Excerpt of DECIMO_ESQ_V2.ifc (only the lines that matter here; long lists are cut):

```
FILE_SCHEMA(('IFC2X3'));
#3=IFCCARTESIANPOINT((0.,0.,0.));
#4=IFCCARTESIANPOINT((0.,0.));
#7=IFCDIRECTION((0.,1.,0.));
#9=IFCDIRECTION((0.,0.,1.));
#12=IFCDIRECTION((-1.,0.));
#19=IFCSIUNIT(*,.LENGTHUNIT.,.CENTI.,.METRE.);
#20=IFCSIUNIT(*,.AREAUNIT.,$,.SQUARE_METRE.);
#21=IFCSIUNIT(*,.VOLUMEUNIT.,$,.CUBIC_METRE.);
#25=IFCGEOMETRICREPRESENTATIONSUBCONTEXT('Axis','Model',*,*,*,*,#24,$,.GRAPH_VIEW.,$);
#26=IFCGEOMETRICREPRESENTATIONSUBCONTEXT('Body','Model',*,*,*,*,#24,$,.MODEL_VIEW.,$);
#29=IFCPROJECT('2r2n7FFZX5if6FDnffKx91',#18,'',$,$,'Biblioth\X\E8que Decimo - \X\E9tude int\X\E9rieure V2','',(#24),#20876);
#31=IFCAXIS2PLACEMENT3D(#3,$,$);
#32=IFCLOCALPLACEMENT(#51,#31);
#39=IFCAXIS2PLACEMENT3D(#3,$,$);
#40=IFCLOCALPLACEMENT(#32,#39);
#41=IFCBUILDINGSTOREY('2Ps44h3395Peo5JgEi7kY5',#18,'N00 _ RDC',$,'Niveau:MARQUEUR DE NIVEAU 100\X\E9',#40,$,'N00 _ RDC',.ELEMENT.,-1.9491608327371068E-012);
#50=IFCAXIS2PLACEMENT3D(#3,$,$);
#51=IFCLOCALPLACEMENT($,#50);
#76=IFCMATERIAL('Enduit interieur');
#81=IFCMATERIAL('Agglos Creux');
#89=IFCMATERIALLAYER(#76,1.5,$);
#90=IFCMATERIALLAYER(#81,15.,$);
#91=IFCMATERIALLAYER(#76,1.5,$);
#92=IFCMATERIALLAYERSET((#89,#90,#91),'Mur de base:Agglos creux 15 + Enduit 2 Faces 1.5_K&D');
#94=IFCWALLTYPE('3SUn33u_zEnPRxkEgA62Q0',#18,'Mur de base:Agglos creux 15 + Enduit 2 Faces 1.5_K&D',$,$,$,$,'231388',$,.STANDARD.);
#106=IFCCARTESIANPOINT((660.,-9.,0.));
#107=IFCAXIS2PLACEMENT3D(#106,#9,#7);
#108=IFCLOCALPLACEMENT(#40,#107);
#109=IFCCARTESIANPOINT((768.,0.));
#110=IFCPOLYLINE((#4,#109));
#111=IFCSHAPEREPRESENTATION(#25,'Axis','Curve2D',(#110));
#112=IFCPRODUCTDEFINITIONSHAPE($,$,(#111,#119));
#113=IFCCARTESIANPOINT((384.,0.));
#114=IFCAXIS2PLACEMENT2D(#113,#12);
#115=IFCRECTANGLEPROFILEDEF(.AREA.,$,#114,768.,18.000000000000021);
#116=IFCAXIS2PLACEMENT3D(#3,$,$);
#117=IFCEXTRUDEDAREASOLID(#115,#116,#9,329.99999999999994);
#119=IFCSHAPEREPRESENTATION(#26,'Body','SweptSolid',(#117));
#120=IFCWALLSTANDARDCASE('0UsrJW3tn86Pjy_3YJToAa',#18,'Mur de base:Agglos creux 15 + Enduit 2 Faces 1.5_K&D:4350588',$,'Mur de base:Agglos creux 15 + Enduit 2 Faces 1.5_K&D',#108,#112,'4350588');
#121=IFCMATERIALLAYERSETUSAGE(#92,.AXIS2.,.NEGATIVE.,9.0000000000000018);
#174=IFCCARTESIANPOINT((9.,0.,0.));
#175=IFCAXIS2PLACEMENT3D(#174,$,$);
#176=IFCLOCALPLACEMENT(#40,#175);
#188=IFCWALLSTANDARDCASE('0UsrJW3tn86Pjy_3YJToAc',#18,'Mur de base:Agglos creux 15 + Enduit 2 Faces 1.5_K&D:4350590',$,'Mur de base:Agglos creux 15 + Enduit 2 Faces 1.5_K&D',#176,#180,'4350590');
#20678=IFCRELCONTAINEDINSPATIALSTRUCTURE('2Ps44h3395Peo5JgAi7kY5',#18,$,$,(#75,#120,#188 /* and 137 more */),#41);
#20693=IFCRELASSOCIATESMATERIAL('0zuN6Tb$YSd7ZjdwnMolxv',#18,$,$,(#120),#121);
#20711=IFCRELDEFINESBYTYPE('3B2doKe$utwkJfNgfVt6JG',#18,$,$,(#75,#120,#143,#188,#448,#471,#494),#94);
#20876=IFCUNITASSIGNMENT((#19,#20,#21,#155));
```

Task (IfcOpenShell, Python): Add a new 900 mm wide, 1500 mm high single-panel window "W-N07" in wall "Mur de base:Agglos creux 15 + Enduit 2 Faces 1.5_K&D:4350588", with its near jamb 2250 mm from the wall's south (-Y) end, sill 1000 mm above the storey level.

```python
import numpy as np
import ifcopenshell
import ifcopenshell.api.feature
import ifcopenshell.api.geometry
import ifcopenshell.api.root
import ifcopenshell.api.spatial
import ifcopenshell.api.type
import ifcopenshell.geom
import ifcopenshell.util.element
import ifcopenshell.util.placement
import ifcopenshell.util.representation
import ifcopenshell.util.shape
import ifcopenshell.util.unit

model = ifcopenshell.open("DECIMO_ESQ_V2.ifc")
unit_scale = ifcopenshell.util.unit.calculate_unit_scale(model)
settings = ifcopenshell.geom.settings()


def volume(element):
    """Net volume in cubic metres, openings subtracted."""
    shape = ifcopenshell.geom.create_shape(settings, element)
    return ifcopenshell.util.shape.get_volume(shape.geometry)


wall = model.by_guid("0UsrJW3tn86Pjy_3YJToAa")
storey = ifcopenshell.util.element.get_container(wall, ifc_class="IfcBuildingStorey")
context = ifcopenshell.util.representation.get_context(model, "Model", "Body", "MODEL_VIEW")
before = volume(wall)

width, height, from_end, sill = 0.9, 1.5, 2.25, 1  # metres

# The wall runs along its own X axis, and the end named is its -X end.
wall_shape = ifcopenshell.geom.create_shape(settings, wall)
x, y, z = ifcopenshell.util.shape.get_vertices(wall_shape.geometry).T
start = x.min() + from_end
face, thickness = float(y.min()), float(y.max() - y.min())
wall_matrix = ifcopenshell.util.placement.get_local_placement(wall.ObjectPlacement)
level = ifcopenshell.util.placement.get_local_placement(storey.ObjectPlacement)[2, 3]


def in_wall(x, y):
    """Placement at x, y metres in the wall's axes, at sill height."""
    matrix = wall_matrix.copy()
    matrix[:, 3] = wall_matrix @ np.array([x / unit_scale, y / unit_scale, 0.0, 1.0])
    matrix[2, 3] = level + sill / unit_scale
    return matrix


# Opening: a box that overshoots both wall faces by 50 mm.
opening = ifcopenshell.api.root.create_entity(model, ifc_class="IfcOpeningElement")
box = ifcopenshell.api.geometry.add_wall_representation(
    model, context=context, length=width, height=height, thickness=thickness + 0.1
)
ifcopenshell.api.geometry.assign_representation(model, product=opening, representation=box)
ifcopenshell.api.geometry.edit_object_placement(model, product=opening, matrix=in_wall(start, face - 0.05), is_si=False)
ifcopenshell.api.feature.add_feature(model, feature=opening, element=wall)

window = ifcopenshell.api.root.create_entity(model, ifc_class="IfcWindow", name="W-N07")
window.OverallWidth, window.OverallHeight = width / unit_scale, height / unit_scale
body = ifcopenshell.api.geometry.add_window_representation(
    model,
    context=context,
    overall_width=window.OverallWidth,
    overall_height=window.OverallHeight,
    partition_type="SINGLE_PANEL",
)
ifcopenshell.api.geometry.assign_representation(model, product=window, representation=body)
ifcopenshell.api.spatial.assign_container(model, products=[window], relating_structure=storey)
fills = ifcopenshell.api.feature.add_filling(model, opening=opening, element=window)
fills.OwnerHistory = window.OwnerHistory  # required in IFC2X3

# IFC2X3 keeps the operation on the window style.
style = ifcopenshell.api.root.create_entity(model, ifc_class="IfcWindowStyle", name="W-N07")
style.OperationType, style.ConstructionType = "SINGLE_PANEL", "NOTDEFINED"
style.ParameterTakesPrecedence = style.Sizeable = False
ifcopenshell.api.type.assign_type(model, related_objects=[window], relating_type=style)

# Centre the window in the wall's thickness.
ifcopenshell.api.geometry.edit_object_placement(model, product=window, matrix=in_wall(start, face), is_si=False)
window_shape = ifcopenshell.geom.create_shape(settings, window)
depth = ifcopenshell.util.shape.get_vertices(window_shape.geometry)[:, 1]
offset = face + thickness / 2 - (depth.min() + depth.max()) / 2
ifcopenshell.api.geometry.edit_object_placement(model, product=window, matrix=in_wall(start, offset), is_si=False)

after = volume(wall)

print(f"wall volume {before:.3f} -> {after:.3f} m3")

model.write("DECIMO_ESQ_V2_v2.ifc")
```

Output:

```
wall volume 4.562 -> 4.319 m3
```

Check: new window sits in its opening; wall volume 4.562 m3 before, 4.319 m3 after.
